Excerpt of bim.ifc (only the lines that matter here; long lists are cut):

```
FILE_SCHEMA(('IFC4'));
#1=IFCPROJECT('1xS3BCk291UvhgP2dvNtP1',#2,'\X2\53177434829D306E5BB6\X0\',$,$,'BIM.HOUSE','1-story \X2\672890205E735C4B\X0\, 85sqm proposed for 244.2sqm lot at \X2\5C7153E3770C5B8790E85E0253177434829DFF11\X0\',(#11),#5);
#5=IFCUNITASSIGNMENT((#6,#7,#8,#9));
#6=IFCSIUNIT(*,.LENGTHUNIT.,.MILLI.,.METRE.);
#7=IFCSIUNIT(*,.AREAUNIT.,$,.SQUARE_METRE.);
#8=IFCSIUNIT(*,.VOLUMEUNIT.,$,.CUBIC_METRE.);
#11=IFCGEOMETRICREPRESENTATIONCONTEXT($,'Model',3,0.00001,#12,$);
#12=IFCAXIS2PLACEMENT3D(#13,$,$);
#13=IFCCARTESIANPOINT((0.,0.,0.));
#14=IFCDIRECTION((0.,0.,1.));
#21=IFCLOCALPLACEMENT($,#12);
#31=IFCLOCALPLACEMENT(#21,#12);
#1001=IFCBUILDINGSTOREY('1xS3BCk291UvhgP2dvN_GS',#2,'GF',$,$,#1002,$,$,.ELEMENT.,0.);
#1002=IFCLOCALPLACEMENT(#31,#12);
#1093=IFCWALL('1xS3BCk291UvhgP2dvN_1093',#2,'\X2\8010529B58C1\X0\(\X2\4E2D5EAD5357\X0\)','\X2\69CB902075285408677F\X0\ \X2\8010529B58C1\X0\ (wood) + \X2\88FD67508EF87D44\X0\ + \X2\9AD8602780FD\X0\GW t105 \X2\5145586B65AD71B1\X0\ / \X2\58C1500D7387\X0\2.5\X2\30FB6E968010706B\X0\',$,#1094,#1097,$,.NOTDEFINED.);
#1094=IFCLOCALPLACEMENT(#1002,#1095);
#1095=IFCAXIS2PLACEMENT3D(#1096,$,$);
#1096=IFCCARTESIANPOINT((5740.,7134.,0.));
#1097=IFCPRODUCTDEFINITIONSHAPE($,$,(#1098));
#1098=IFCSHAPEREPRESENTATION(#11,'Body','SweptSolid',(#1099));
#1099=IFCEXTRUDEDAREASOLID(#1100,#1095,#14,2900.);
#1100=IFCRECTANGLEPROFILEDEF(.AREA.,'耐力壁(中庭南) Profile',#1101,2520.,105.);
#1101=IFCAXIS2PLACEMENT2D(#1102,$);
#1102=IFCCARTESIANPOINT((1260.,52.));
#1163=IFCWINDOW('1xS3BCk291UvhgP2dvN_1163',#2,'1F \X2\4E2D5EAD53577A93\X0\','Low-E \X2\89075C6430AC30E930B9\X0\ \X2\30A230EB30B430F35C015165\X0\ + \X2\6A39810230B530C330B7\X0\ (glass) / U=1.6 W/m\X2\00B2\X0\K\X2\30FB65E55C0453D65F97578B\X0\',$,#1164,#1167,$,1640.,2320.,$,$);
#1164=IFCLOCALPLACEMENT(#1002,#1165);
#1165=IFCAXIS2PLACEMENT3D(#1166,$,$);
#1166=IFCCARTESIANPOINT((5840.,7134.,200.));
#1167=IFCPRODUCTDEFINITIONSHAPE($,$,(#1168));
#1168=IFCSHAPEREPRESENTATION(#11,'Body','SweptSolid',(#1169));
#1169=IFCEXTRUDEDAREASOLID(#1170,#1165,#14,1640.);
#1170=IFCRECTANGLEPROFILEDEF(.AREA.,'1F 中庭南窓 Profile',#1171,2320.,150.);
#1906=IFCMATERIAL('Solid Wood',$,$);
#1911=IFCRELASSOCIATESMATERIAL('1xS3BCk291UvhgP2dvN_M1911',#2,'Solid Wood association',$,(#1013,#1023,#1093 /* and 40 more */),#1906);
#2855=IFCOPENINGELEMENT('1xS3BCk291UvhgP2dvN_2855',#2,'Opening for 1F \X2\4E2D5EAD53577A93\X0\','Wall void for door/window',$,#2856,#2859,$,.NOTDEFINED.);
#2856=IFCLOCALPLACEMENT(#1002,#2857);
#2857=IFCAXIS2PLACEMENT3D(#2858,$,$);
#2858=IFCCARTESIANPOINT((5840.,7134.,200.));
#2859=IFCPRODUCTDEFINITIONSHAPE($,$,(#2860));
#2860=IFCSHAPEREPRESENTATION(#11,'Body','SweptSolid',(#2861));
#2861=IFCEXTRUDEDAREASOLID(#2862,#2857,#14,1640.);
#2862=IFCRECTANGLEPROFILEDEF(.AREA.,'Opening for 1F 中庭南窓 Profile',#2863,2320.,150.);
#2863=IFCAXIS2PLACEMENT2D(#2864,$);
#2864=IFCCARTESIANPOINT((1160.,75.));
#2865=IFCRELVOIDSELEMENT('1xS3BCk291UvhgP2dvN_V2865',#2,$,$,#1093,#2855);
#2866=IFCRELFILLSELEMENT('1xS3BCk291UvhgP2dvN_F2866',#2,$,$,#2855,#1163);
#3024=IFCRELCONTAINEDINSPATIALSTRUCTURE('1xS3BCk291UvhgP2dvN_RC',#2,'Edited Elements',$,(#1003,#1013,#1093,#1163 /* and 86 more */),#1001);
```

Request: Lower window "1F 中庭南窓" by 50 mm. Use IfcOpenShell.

```python
import numpy as np
import ifcopenshell
import ifcopenshell.api.geometry
import ifcopenshell.util.placement
import ifcopenshell.util.unit

model = ifcopenshell.open("bim.ifc")
unit_scale = ifcopenshell.util.unit.calculate_unit_scale(model)

window = model.by_guid("1xS3BCk291UvhgP2dvN_1163")
opening = window.FillsVoids[0].RelatingOpeningElement
dz = -0.05 / unit_scale

shift = np.array([0.0, 0.0, dz])
# The window is not placed relative to its opening, so move both.
for product in (opening, window):
    matrix = ifcopenshell.util.placement.get_local_placement(product.ObjectPlacement)
    matrix[:3, 3] += shift
    ifcopenshell.api.geometry.edit_object_placement(model, product=product, matrix=matrix, is_si=False)

print(f"moved by {dz * unit_scale:+.3f} m")

model.write("bim_updated.ifc")
```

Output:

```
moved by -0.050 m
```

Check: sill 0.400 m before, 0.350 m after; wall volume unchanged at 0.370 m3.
